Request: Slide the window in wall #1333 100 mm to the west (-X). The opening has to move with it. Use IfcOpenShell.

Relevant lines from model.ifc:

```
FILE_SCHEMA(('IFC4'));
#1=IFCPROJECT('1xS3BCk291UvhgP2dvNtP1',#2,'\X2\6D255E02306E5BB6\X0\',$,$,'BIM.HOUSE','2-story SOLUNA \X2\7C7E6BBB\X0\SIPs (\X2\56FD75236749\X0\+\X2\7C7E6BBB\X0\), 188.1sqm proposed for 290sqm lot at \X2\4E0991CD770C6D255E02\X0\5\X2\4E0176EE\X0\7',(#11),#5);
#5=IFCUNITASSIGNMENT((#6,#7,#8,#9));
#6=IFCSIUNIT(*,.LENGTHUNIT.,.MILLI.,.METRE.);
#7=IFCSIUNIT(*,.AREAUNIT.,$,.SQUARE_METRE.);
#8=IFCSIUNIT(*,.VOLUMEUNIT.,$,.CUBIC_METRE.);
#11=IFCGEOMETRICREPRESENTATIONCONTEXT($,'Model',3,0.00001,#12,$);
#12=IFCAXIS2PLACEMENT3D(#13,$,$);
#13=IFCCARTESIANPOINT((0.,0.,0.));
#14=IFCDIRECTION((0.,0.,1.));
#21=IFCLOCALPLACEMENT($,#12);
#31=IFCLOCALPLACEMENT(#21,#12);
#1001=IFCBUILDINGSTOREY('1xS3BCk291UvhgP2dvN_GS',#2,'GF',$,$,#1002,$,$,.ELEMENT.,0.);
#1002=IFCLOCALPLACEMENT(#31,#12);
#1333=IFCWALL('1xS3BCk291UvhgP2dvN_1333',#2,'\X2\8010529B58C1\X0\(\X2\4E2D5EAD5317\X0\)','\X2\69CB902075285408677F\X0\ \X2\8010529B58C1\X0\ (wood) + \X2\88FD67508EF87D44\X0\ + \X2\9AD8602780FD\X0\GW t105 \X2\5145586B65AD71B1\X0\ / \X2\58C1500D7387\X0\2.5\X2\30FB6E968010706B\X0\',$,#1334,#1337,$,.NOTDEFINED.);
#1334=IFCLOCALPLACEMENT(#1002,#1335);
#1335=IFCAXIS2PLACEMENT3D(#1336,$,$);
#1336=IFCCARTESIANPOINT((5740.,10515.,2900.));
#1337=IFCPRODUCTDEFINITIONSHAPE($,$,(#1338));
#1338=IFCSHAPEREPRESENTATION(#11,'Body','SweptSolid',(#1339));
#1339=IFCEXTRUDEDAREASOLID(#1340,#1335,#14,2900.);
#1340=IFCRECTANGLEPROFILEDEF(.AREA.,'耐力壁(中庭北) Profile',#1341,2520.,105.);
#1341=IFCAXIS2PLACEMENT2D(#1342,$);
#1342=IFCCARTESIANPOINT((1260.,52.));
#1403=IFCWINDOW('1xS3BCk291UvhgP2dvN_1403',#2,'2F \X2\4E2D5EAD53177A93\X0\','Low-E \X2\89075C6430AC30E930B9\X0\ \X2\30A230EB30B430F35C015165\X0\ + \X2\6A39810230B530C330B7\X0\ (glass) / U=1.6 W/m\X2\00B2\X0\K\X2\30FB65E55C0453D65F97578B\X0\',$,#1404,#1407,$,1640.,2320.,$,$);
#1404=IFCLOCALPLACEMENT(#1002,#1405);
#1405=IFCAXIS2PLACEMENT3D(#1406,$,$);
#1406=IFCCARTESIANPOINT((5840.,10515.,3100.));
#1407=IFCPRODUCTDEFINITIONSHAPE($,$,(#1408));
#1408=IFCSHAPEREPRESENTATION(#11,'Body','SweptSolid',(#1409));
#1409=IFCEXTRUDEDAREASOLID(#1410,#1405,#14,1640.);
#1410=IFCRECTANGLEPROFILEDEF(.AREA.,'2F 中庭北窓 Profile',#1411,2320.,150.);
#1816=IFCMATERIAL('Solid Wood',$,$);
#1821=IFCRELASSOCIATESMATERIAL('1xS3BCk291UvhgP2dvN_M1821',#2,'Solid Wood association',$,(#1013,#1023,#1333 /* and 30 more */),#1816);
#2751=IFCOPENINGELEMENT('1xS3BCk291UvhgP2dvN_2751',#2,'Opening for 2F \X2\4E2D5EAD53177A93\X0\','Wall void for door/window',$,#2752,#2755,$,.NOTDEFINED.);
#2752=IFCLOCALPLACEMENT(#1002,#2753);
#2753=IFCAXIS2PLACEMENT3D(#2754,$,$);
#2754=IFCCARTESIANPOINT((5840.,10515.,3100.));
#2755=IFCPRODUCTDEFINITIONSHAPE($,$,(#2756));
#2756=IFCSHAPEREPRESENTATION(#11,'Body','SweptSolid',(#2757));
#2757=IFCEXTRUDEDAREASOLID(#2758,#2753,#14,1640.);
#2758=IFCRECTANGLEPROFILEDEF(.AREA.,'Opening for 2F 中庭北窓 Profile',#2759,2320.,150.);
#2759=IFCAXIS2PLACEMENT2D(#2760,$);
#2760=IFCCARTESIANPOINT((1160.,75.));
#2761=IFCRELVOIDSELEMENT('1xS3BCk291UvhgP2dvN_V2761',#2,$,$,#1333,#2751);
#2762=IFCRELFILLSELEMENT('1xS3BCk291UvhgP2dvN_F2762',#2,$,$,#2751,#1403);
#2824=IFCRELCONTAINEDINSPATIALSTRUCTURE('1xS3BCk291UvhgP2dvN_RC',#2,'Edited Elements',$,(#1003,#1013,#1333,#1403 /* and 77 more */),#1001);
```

```python
import ifcopenshell
import ifcopenshell.api.geometry
import ifcopenshell.util.placement
import ifcopenshell.util.unit

model = ifcopenshell.open("model.ifc")
unit_scale = ifcopenshell.util.unit.calculate_unit_scale(model)

window = model.by_id(1403)
opening = window.FillsVoids[0].RelatingOpeningElement
wall = opening.VoidsElements[0].RelatingBuildingElement

wall_matrix = ifcopenshell.util.placement.get_local_placement(wall.ObjectPlacement)
shift = wall_matrix[:3, 0] * -0.1 / unit_scale
before = ifcopenshell.util.placement.get_local_placement(window.ObjectPlacement)[:3, 3].copy()

# The window is not placed relative to its opening, so move both.
for product in (opening, window):
    matrix = ifcopenshell.util.placement.get_local_placement(product.ObjectPlacement)
    matrix[:3, 3] += shift
    ifcopenshell.api.geometry.edit_object_placement(model, product=product, matrix=matrix, is_si=False)

after = ifcopenshell.util.placement.get_local_placement(window.ObjectPlacement)[:3, 3]
print("window moved by", (after - before).round(3) + 0.0)

model.write("model_edited.ifc")
```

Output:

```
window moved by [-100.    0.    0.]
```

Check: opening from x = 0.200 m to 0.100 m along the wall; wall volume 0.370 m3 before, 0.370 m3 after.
